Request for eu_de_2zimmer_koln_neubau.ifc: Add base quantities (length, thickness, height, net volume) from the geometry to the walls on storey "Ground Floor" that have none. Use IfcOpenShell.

First a look at what the model holds.

```python
import ifcopenshell
import ifcopenshell.util.element
import ifcopenshell.util.unit

model = ifcopenshell.open("eu_de_2zimmer_koln_neubau.ifc")
print(model.schema)
for unit_type in ("LENGTHUNIT", "AREAUNIT", "VOLUMEUNIT"):
    print(unit_type, ifcopenshell.util.unit.calculate_unit_scale(model, unit_type))
storey = next(s for s in model.by_type("IfcBuildingStorey") if s.Name == "Ground Floor")
walls = [e for e in ifcopenshell.util.element.get_decomposition(storey) if e.is_a("IfcWall")]
for e in sorted(walls, key=lambda e: e.id()):
    print(e.id(), e.is_a(), e.Name, list(ifcopenshell.util.element.get_psets(e, qtos_only=True)), sep=" | ")
```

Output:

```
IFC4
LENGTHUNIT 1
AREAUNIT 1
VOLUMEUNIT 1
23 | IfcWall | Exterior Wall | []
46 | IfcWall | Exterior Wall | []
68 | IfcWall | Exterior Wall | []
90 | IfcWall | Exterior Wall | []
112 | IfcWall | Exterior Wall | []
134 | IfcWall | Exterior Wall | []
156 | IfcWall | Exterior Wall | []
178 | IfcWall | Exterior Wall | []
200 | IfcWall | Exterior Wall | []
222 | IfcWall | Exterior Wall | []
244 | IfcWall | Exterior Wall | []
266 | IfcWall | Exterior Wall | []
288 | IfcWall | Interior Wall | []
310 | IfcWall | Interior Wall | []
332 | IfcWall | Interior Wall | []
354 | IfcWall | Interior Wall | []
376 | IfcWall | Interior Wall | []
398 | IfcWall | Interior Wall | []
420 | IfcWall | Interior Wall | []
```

```python
import ifcopenshell
import ifcopenshell.api.pset
import ifcopenshell.geom
import ifcopenshell.util.element
import ifcopenshell.util.shape
import ifcopenshell.util.unit

model = ifcopenshell.open("eu_de_2zimmer_koln_neubau.ifc")
unit_scale = ifcopenshell.util.unit.calculate_unit_scale(model)
volume_scale = ifcopenshell.util.unit.calculate_unit_scale(model, "VOLUMEUNIT")
settings = ifcopenshell.geom.settings()

storey = next(s for s in model.by_type("IfcBuildingStorey") if s.Name == "Ground Floor")
walls = [e for e in ifcopenshell.util.element.get_decomposition(storey) if e.is_a("IfcWall")]

for e in sorted(walls, key=lambda e: e.id()):
    if ifcopenshell.util.element.get_psets(e, qtos_only=True, should_inherit=False):
        continue
    # Geometry comes back in metres, in the element's own axes.
    shape = ifcopenshell.geom.create_shape(settings, e)
    values = {
        "Length": ifcopenshell.util.shape.get_x(shape.geometry) / unit_scale,
        "Width": ifcopenshell.util.shape.get_y(shape.geometry) / unit_scale,
        "Height": ifcopenshell.util.shape.get_z(shape.geometry) / unit_scale,
        "NetVolume": ifcopenshell.util.shape.get_volume(shape.geometry) / volume_scale,
    }
    qto = ifcopenshell.api.pset.add_qto(model, product=e, name="Qto_WallBaseQuantities")
    ifcopenshell.api.pset.edit_qto(model, qto=qto, properties=values)
    print(e.id(), {k: round(v, 3) for k, v in values.items()})

model.write("eu_de_2zimmer_koln_neubau_v2.ifc")
```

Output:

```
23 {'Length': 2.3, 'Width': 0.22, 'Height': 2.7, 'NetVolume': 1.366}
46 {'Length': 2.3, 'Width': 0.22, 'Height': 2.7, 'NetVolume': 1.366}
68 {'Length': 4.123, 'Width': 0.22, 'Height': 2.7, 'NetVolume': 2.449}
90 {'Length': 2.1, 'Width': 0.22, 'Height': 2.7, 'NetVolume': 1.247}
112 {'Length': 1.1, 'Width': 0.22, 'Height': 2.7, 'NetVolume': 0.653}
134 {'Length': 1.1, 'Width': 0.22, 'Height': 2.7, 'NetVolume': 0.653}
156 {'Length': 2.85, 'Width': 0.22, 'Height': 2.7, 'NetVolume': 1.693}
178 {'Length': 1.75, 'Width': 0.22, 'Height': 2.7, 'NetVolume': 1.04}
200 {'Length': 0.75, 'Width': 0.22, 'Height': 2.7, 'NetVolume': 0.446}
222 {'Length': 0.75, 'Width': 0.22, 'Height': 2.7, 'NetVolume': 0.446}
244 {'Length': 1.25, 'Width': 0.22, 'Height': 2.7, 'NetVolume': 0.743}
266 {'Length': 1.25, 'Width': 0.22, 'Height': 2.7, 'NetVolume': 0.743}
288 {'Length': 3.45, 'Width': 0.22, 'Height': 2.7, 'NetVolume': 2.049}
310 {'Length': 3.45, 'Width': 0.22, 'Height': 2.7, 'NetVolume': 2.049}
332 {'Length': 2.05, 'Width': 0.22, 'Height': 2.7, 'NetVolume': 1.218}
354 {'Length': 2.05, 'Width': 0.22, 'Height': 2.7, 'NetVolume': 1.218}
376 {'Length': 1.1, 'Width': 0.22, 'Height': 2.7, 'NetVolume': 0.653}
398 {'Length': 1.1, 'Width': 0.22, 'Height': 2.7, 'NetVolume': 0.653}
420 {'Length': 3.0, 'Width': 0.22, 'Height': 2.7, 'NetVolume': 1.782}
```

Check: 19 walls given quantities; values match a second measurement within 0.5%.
